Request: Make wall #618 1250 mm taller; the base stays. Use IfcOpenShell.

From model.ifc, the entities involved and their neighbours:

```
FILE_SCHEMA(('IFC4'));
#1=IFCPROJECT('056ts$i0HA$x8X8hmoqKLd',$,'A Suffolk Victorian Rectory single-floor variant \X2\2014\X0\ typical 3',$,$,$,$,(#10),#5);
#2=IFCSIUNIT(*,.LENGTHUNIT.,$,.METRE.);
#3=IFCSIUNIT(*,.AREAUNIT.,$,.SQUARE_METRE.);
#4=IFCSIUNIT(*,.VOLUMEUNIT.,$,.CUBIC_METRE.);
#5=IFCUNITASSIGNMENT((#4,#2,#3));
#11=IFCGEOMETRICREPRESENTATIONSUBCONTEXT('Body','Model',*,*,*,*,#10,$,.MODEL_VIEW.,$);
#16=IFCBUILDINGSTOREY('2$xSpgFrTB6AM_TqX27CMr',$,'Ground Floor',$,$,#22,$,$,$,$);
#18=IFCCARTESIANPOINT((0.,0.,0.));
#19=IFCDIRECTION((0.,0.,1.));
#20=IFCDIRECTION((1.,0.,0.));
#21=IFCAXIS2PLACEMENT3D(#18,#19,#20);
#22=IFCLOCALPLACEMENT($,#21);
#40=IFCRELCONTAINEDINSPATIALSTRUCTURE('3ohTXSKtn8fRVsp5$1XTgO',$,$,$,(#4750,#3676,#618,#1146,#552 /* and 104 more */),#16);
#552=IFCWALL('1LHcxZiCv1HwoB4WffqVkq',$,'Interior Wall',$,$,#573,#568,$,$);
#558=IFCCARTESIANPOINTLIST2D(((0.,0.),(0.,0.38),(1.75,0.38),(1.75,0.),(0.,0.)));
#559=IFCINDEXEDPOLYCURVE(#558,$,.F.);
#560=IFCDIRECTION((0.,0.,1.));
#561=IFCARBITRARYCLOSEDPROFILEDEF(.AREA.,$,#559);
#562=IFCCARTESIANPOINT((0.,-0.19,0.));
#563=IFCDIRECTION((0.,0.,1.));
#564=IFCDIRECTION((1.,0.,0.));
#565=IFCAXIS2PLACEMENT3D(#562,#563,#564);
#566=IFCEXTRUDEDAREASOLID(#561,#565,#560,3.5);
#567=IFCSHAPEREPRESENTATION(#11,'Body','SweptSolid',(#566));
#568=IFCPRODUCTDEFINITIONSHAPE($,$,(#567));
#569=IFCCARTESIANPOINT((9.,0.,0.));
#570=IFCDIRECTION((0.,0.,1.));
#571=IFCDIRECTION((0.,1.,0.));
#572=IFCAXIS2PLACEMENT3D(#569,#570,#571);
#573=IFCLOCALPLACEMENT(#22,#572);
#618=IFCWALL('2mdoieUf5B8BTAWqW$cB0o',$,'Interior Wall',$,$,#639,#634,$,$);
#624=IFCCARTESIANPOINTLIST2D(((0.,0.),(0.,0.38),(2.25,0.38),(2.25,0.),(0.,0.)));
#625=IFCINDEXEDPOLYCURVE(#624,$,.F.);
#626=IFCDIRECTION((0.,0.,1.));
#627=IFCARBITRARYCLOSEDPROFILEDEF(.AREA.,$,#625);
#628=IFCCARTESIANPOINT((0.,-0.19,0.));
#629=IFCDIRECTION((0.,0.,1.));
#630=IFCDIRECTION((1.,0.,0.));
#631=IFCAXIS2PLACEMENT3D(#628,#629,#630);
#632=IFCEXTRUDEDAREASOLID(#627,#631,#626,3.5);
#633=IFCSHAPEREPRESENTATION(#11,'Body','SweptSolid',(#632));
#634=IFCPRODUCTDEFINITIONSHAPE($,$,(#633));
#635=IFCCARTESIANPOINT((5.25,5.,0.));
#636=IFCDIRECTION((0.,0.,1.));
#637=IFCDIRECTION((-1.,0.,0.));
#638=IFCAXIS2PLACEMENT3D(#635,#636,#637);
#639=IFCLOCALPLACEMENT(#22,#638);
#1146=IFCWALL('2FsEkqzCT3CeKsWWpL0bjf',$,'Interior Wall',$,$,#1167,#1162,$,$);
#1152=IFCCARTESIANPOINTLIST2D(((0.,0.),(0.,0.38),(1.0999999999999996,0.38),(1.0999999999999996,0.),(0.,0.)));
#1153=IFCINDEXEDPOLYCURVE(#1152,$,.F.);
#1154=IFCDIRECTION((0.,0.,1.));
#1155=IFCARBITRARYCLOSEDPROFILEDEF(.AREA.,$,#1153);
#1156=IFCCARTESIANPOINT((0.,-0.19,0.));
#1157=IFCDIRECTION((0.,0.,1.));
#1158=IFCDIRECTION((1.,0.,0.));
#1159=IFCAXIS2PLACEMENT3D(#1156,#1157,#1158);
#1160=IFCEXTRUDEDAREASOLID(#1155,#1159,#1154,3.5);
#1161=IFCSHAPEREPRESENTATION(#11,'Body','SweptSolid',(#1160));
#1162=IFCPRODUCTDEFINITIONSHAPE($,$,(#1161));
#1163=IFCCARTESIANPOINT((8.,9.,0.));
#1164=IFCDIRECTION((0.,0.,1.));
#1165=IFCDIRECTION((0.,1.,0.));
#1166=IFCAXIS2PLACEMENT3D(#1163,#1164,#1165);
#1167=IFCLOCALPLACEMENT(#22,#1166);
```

```python
import ifcopenshell
import ifcopenshell.geom
import ifcopenshell.util.representation
import ifcopenshell.util.shape
import ifcopenshell.util.unit

model = ifcopenshell.open("model.ifc")
unit_scale = ifcopenshell.util.unit.calculate_unit_scale(model)
settings = ifcopenshell.geom.settings()


def volume(element):
    """Net volume in cubic metres, openings subtracted."""
    shape = ifcopenshell.geom.create_shape(settings, element)
    return ifcopenshell.util.shape.get_volume(shape.geometry)


wall = model.by_guid("2mdoieUf5B8BTAWqW$cB0o")
before = volume(wall)

body = ifcopenshell.util.representation.get_representation(wall, "Model", "Body")
solid = body.Items[0]
old_height = solid.Depth
solid.Depth += 1.25 / unit_scale
after = volume(wall)

print(f"height {old_height:g} -> {solid.Depth:g}, volume {before:.3f} -> {after:.3f} m3")

model.write("model_edited.ifc")
```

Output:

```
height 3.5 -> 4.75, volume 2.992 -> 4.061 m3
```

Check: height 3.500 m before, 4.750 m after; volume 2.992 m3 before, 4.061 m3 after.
